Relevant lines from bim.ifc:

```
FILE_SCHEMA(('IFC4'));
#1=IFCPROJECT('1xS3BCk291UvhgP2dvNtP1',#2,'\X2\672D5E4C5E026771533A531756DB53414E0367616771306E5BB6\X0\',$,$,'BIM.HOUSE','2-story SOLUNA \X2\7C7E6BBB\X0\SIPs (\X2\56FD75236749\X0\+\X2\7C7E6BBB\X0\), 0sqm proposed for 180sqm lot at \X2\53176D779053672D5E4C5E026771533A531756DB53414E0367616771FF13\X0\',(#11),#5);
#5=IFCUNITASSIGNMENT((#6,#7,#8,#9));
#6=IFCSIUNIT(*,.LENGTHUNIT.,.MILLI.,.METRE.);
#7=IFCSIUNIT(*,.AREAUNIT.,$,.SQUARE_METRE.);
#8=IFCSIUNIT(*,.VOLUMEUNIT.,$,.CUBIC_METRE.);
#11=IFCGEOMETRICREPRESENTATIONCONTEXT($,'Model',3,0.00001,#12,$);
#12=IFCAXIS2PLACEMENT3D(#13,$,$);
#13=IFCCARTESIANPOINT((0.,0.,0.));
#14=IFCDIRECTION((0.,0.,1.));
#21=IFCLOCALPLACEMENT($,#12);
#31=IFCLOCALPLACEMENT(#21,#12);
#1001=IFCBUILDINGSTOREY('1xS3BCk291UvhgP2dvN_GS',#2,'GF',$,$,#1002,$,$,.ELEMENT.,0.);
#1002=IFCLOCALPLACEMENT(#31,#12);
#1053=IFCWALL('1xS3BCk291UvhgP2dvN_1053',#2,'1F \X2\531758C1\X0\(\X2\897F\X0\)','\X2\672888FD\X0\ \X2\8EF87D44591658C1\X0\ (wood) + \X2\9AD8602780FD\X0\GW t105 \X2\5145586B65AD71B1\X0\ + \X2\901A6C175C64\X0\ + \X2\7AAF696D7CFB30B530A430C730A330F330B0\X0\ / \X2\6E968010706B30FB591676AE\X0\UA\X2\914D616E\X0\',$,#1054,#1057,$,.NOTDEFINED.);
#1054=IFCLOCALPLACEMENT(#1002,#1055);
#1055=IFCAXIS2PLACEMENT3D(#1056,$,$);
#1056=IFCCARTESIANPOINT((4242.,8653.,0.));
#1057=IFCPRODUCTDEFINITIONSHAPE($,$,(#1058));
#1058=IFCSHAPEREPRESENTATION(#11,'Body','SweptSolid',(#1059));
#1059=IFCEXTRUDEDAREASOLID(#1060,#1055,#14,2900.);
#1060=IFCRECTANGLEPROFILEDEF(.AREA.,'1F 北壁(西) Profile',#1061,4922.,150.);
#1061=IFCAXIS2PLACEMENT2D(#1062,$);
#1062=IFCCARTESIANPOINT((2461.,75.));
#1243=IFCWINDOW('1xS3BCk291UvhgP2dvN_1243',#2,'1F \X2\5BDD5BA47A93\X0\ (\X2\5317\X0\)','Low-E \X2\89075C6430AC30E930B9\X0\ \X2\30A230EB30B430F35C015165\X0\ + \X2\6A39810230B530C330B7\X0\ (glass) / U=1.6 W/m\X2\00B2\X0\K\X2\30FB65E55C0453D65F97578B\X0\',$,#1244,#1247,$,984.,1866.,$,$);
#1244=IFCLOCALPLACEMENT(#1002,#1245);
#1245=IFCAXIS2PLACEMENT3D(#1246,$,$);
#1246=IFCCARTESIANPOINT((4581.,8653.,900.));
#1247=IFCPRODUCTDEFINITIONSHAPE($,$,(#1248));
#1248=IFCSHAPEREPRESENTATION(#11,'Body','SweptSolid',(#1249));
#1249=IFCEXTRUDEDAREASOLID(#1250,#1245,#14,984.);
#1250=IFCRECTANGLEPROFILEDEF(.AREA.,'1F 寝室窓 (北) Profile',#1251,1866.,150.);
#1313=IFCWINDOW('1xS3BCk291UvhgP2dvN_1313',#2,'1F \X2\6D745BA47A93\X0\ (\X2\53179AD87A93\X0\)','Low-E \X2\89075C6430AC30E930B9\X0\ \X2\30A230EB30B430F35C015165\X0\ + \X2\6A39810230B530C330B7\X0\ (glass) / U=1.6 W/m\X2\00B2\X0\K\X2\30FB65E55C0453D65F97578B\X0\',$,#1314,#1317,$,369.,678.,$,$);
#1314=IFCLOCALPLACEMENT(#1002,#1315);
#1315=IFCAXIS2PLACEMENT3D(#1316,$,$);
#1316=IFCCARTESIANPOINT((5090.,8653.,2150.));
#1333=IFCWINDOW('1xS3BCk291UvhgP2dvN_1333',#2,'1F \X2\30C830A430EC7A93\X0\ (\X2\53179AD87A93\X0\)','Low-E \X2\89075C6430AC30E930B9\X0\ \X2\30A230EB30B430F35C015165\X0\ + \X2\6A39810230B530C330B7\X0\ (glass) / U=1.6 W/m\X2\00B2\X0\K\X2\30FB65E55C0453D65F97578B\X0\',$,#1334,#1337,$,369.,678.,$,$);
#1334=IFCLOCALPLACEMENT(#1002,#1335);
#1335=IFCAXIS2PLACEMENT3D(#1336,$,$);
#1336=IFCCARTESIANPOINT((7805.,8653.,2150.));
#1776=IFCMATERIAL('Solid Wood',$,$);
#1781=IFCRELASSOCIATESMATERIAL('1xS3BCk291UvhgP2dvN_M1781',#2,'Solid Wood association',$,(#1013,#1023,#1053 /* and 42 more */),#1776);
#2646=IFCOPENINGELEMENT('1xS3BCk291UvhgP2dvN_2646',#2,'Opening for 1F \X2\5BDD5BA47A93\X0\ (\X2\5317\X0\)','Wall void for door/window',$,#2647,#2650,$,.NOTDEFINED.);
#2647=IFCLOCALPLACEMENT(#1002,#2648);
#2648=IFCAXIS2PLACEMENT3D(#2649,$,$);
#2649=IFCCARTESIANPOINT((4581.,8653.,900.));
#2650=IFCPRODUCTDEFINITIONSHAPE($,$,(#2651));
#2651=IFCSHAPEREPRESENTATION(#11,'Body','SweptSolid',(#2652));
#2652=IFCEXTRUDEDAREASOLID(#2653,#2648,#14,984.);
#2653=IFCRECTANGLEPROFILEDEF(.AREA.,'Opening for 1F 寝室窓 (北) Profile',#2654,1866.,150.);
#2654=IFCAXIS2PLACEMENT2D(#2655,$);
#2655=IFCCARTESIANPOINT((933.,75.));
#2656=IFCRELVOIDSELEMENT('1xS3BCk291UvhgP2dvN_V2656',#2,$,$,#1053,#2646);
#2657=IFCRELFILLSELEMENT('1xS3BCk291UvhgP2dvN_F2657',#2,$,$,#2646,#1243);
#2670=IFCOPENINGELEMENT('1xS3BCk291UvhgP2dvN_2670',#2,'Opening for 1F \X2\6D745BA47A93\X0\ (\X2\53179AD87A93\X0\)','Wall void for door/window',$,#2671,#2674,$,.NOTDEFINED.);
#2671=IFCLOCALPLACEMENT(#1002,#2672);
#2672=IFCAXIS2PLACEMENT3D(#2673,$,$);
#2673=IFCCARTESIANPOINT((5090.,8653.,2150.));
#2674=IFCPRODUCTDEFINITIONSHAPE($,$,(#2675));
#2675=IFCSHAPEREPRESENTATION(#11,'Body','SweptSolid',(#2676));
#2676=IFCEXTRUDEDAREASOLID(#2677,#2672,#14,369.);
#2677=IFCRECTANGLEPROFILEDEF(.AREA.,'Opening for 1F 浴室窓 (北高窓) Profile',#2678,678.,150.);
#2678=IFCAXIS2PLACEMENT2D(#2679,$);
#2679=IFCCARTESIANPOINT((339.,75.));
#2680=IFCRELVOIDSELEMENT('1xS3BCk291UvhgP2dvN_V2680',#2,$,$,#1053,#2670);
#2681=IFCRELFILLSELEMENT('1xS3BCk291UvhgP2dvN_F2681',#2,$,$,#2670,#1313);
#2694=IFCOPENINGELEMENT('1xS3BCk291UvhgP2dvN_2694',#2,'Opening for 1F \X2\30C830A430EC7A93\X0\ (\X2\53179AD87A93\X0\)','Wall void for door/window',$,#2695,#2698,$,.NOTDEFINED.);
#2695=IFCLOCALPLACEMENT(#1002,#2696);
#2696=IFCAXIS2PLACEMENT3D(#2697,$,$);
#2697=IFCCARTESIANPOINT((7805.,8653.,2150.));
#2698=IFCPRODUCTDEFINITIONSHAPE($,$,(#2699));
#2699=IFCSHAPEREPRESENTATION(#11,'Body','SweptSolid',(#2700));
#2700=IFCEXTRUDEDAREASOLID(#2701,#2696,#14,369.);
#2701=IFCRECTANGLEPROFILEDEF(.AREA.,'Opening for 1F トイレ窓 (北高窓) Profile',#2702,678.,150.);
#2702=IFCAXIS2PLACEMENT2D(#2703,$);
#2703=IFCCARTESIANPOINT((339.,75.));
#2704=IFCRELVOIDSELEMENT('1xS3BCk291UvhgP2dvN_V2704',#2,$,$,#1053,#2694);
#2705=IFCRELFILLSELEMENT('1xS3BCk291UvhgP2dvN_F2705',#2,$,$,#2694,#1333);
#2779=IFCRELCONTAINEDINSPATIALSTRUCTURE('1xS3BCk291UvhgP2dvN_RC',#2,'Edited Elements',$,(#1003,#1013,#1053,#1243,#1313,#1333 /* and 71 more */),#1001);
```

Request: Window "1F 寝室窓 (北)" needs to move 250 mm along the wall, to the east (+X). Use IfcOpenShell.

```python
import ifcopenshell
import ifcopenshell.api.geometry
import ifcopenshell.util.placement
import ifcopenshell.util.unit

model = ifcopenshell.open("bim.ifc")
unit_scale = ifcopenshell.util.unit.calculate_unit_scale(model)

window = model.by_guid("1xS3BCk291UvhgP2dvN_1243")
opening = window.FillsVoids[0].RelatingOpeningElement
wall = opening.VoidsElements[0].RelatingBuildingElement

wall_matrix = ifcopenshell.util.placement.get_local_placement(wall.ObjectPlacement)
shift = wall_matrix[:3, 0] * 0.25 / unit_scale
before = ifcopenshell.util.placement.get_local_placement(window.ObjectPlacement)[:3, 3].copy()

# The window is not placed relative to its opening, so move both.
for product in (opening, window):
    matrix = ifcopenshell.util.placement.get_local_placement(product.ObjectPlacement)
    matrix[:3, 3] += shift
    ifcopenshell.api.geometry.edit_object_placement(model, product=product, matrix=matrix, is_si=False)

after = ifcopenshell.util.placement.get_local_placement(window.ObjectPlacement)[:3, 3]
print("window moved by", (after - before).round(3) + 0.0)

model.write("bim_updated.ifc")
```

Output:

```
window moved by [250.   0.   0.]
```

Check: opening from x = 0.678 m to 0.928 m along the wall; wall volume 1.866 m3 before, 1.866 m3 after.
